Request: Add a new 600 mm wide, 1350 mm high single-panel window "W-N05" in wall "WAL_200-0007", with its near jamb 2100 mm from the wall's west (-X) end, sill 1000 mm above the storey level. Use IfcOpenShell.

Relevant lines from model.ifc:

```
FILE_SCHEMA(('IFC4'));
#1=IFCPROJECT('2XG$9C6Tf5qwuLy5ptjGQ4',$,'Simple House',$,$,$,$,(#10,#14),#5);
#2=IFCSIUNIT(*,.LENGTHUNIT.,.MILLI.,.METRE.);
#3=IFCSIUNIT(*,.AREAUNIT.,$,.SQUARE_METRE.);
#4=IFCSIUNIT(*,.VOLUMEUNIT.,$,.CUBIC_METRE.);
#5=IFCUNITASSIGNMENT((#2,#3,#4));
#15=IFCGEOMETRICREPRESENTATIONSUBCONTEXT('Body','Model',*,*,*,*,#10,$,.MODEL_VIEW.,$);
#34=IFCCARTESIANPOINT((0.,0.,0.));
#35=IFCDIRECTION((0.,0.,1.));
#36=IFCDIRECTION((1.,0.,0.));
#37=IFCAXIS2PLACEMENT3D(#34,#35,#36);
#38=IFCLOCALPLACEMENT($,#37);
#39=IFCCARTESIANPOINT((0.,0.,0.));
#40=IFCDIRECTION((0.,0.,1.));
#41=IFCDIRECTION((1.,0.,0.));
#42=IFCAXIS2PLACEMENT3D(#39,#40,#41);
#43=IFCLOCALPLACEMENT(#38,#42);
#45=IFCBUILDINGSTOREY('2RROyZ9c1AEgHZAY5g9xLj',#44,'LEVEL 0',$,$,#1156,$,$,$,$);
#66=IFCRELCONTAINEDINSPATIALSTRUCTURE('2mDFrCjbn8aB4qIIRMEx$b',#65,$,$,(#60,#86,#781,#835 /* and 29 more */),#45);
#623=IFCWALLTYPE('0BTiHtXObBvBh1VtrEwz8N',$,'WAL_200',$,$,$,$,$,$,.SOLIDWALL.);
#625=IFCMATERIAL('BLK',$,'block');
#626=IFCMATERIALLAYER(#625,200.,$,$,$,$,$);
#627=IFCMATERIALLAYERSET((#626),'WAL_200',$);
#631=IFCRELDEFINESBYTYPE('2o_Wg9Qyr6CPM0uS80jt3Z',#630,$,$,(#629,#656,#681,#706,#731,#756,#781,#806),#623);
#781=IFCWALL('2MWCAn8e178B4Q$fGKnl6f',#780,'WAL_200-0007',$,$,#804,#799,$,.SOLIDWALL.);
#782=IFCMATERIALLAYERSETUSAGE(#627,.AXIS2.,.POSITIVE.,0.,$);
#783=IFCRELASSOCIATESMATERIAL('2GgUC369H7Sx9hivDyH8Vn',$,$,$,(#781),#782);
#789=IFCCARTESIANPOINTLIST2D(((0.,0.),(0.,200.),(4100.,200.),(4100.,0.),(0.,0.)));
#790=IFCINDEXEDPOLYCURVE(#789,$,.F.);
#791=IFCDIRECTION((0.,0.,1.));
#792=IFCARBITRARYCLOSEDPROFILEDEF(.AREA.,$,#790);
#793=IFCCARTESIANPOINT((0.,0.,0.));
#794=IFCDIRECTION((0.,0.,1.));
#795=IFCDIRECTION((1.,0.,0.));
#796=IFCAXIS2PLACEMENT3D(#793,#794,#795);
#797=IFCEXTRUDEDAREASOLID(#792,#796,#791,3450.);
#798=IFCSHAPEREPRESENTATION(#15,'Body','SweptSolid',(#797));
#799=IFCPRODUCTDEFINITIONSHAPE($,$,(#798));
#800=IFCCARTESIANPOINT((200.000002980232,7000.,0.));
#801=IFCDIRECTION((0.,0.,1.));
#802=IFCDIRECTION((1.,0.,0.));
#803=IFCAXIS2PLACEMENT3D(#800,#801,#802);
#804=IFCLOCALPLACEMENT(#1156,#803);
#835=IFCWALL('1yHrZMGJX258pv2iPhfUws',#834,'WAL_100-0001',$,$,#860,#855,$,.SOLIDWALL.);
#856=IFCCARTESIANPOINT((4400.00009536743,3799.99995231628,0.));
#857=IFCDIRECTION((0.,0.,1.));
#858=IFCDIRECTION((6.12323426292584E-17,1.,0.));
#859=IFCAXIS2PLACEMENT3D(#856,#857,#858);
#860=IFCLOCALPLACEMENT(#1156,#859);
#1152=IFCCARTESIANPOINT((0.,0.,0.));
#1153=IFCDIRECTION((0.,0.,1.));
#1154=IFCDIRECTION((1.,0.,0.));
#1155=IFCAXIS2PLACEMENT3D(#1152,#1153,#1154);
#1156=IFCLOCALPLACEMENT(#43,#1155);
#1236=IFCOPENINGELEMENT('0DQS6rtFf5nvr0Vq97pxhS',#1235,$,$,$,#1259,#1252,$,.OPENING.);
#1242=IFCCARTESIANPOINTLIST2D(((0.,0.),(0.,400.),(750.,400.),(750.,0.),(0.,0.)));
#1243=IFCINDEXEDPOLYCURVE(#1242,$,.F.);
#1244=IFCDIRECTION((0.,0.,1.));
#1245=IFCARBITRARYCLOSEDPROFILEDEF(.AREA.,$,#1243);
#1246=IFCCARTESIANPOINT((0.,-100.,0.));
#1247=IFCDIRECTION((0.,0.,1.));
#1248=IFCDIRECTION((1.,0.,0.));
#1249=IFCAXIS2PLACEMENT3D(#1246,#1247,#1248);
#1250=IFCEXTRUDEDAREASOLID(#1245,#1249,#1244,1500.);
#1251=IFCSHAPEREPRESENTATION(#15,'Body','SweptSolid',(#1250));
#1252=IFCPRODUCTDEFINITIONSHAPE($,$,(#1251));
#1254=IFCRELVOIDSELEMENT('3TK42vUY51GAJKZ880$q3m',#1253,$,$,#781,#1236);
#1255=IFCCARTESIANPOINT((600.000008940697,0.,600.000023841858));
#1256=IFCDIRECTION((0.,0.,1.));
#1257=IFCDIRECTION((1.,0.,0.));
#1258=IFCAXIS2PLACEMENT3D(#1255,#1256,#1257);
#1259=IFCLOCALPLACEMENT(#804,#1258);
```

```python
import numpy as np
import ifcopenshell
import ifcopenshell.api.feature
import ifcopenshell.api.geometry
import ifcopenshell.api.root
import ifcopenshell.api.spatial
import ifcopenshell.geom
import ifcopenshell.util.element
import ifcopenshell.util.placement
import ifcopenshell.util.representation
import ifcopenshell.util.shape
import ifcopenshell.util.unit

model = ifcopenshell.open("model.ifc")
unit_scale = ifcopenshell.util.unit.calculate_unit_scale(model)
settings = ifcopenshell.geom.settings()


def volume(element):
    """Net volume in cubic metres, openings subtracted."""
    shape = ifcopenshell.geom.create_shape(settings, element)
    return ifcopenshell.util.shape.get_volume(shape.geometry)


wall = model.by_id(781)
storey = ifcopenshell.util.element.get_container(wall, ifc_class="IfcBuildingStorey")
context = ifcopenshell.util.representation.get_context(model, "Model", "Body", "MODEL_VIEW")
before = volume(wall)

width, height, from_end, sill = 0.6, 1.35, 2.1, 1  # metres

# The wall runs along its own X axis, and the end named is its -X end.
wall_shape = ifcopenshell.geom.create_shape(settings, wall)
x, y, z = ifcopenshell.util.shape.get_vertices(wall_shape.geometry).T
start = x.min() + from_end
face, thickness = float(y.min()), float(y.max() - y.min())
wall_matrix = ifcopenshell.util.placement.get_local_placement(wall.ObjectPlacement)
level = ifcopenshell.util.placement.get_local_placement(storey.ObjectPlacement)[2, 3]


def in_wall(x, y):
    """Placement at x, y metres in the wall's axes, at sill height."""
    matrix = wall_matrix.copy()
    matrix[:, 3] = wall_matrix @ np.array([x / unit_scale, y / unit_scale, 0.0, 1.0])
    matrix[2, 3] = level + sill / unit_scale
    return matrix


# Opening: a box that overshoots both wall faces by 50 mm.
opening = ifcopenshell.api.root.create_entity(model, ifc_class="IfcOpeningElement", predefined_type="OPENING")
box = ifcopenshell.api.geometry.add_wall_representation(
    model, context=context, length=width, height=height, thickness=thickness + 0.1
)
ifcopenshell.api.geometry.assign_representation(model, product=opening, representation=box)
ifcopenshell.api.geometry.edit_object_placement(model, product=opening, matrix=in_wall(start, face - 0.05), is_si=False)
ifcopenshell.api.feature.add_feature(model, feature=opening, element=wall)

window = ifcopenshell.api.root.create_entity(model, ifc_class="IfcWindow", name="W-N05", predefined_type="WINDOW")
window.OverallWidth, window.OverallHeight = width / unit_scale, height / unit_scale
window.PartitioningType = "SINGLE_PANEL"
body = ifcopenshell.api.geometry.add_window_representation(
    model,
    context=context,
    overall_width=window.OverallWidth,
    overall_height=window.OverallHeight,
    partition_type="SINGLE_PANEL",
)
ifcopenshell.api.geometry.assign_representation(model, product=window, representation=body)
ifcopenshell.api.spatial.assign_container(model, products=[window], relating_structure=storey)
ifcopenshell.api.feature.add_filling(model, opening=opening, element=window)

# Centre the window in the wall's thickness.
ifcopenshell.api.geometry.edit_object_placement(model, product=window, matrix=in_wall(start, face), is_si=False)
window_shape = ifcopenshell.geom.create_shape(settings, window)
depth = ifcopenshell.util.shape.get_vertices(window_shape.geometry)[:, 1]
offset = face + thickness / 2 - (depth.min() + depth.max()) / 2
ifcopenshell.api.geometry.edit_object_placement(model, product=window, matrix=in_wall(start, offset), is_si=False)

after = volume(wall)

print(f"wall volume {before:.3f} -> {after:.3f} m3")

model.write("model_rev.ifc")
```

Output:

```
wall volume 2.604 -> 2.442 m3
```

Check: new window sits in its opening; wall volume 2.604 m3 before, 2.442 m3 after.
